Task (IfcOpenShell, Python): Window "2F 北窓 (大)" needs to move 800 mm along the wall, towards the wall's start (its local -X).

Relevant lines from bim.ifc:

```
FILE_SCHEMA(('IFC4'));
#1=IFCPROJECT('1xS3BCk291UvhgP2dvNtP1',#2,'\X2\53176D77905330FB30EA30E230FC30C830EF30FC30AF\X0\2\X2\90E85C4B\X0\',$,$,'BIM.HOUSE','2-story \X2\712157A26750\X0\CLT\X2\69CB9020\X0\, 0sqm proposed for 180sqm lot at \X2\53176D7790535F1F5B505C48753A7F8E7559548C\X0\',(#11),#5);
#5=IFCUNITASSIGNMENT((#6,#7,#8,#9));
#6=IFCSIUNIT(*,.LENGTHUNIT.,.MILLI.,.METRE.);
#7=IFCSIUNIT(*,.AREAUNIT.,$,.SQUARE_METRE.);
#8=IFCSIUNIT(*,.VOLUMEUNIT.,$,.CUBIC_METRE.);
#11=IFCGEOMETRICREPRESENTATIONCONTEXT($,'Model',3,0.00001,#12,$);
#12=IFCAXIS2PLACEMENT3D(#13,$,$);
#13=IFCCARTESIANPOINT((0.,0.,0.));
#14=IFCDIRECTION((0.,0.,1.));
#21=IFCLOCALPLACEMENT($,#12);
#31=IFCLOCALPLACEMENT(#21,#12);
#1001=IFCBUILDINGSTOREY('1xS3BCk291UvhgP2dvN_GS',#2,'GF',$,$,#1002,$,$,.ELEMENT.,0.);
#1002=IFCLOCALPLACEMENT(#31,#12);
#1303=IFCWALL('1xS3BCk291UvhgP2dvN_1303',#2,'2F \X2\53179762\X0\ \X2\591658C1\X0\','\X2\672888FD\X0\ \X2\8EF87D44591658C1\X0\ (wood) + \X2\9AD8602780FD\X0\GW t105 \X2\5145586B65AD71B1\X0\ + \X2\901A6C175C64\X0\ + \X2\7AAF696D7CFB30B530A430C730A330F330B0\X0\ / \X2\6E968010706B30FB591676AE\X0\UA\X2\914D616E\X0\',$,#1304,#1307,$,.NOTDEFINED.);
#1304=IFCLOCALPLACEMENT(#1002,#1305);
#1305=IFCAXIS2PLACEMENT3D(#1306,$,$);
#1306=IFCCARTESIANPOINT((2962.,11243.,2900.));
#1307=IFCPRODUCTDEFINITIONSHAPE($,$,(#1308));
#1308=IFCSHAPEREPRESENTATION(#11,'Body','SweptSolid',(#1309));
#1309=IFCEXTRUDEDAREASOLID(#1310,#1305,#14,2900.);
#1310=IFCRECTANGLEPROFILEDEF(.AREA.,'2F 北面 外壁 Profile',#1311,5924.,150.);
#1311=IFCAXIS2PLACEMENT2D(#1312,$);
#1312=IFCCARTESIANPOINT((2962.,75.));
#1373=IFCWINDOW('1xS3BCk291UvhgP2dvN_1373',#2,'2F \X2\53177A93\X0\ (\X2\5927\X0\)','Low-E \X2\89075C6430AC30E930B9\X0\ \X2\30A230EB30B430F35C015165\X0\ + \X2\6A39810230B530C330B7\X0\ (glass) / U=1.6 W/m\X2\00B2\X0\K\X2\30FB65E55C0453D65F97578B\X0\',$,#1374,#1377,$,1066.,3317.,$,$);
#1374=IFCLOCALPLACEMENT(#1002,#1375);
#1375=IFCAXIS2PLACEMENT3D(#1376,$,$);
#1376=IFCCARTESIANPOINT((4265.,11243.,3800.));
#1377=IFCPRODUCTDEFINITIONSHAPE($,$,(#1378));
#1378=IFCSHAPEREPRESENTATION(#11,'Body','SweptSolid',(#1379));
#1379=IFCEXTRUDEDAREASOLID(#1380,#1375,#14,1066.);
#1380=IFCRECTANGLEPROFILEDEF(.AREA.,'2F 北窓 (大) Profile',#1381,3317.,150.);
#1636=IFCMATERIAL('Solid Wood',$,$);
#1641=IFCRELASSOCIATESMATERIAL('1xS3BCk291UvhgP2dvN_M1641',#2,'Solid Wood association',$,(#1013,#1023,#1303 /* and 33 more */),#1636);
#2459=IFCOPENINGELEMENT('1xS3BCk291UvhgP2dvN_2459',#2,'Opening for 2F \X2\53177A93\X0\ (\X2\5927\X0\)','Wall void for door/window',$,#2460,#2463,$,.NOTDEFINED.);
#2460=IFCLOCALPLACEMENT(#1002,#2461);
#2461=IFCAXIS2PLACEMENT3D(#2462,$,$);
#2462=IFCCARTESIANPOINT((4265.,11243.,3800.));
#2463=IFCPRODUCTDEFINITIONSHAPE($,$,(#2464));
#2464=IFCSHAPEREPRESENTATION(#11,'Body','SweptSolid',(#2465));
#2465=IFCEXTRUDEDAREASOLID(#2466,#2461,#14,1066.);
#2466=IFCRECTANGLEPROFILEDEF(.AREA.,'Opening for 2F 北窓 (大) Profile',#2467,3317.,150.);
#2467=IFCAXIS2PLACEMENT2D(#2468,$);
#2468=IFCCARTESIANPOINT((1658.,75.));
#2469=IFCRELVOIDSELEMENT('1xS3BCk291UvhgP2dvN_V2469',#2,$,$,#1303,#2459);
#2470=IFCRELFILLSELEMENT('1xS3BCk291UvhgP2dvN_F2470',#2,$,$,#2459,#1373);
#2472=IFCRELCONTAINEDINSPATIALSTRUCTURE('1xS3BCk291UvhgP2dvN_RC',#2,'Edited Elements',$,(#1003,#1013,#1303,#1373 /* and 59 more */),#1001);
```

```python
import ifcopenshell
import ifcopenshell.api.geometry
import ifcopenshell.util.placement

model = ifcopenshell.open("bim.ifc")

window = model.by_guid("1xS3BCk291UvhgP2dvN_1373")
opening = window.FillsVoids[0].RelatingOpeningElement
wall = opening.VoidsElements[0].RelatingBuildingElement

wall_matrix = ifcopenshell.util.placement.get_local_placement(wall.ObjectPlacement)
shift = wall_matrix[:3, 0] * -800.0
before = ifcopenshell.util.placement.get_local_placement(window.ObjectPlacement)[:3, 3].copy()

# The window is not placed relative to its opening, so move both.
for product in (opening, window):
    matrix = ifcopenshell.util.placement.get_local_placement(product.ObjectPlacement)
    matrix[:3, 3] += shift
    ifcopenshell.api.geometry.edit_object_placement(model, product=product, matrix=matrix, is_si=False)

after = ifcopenshell.util.placement.get_local_placement(window.ObjectPlacement)[:3, 3]
print("window moved by", (after - before).round(3) + 0.0)

model.write("bim_rev.ifc")
```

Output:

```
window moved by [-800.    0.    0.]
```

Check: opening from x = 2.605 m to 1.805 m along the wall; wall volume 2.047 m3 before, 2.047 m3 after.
